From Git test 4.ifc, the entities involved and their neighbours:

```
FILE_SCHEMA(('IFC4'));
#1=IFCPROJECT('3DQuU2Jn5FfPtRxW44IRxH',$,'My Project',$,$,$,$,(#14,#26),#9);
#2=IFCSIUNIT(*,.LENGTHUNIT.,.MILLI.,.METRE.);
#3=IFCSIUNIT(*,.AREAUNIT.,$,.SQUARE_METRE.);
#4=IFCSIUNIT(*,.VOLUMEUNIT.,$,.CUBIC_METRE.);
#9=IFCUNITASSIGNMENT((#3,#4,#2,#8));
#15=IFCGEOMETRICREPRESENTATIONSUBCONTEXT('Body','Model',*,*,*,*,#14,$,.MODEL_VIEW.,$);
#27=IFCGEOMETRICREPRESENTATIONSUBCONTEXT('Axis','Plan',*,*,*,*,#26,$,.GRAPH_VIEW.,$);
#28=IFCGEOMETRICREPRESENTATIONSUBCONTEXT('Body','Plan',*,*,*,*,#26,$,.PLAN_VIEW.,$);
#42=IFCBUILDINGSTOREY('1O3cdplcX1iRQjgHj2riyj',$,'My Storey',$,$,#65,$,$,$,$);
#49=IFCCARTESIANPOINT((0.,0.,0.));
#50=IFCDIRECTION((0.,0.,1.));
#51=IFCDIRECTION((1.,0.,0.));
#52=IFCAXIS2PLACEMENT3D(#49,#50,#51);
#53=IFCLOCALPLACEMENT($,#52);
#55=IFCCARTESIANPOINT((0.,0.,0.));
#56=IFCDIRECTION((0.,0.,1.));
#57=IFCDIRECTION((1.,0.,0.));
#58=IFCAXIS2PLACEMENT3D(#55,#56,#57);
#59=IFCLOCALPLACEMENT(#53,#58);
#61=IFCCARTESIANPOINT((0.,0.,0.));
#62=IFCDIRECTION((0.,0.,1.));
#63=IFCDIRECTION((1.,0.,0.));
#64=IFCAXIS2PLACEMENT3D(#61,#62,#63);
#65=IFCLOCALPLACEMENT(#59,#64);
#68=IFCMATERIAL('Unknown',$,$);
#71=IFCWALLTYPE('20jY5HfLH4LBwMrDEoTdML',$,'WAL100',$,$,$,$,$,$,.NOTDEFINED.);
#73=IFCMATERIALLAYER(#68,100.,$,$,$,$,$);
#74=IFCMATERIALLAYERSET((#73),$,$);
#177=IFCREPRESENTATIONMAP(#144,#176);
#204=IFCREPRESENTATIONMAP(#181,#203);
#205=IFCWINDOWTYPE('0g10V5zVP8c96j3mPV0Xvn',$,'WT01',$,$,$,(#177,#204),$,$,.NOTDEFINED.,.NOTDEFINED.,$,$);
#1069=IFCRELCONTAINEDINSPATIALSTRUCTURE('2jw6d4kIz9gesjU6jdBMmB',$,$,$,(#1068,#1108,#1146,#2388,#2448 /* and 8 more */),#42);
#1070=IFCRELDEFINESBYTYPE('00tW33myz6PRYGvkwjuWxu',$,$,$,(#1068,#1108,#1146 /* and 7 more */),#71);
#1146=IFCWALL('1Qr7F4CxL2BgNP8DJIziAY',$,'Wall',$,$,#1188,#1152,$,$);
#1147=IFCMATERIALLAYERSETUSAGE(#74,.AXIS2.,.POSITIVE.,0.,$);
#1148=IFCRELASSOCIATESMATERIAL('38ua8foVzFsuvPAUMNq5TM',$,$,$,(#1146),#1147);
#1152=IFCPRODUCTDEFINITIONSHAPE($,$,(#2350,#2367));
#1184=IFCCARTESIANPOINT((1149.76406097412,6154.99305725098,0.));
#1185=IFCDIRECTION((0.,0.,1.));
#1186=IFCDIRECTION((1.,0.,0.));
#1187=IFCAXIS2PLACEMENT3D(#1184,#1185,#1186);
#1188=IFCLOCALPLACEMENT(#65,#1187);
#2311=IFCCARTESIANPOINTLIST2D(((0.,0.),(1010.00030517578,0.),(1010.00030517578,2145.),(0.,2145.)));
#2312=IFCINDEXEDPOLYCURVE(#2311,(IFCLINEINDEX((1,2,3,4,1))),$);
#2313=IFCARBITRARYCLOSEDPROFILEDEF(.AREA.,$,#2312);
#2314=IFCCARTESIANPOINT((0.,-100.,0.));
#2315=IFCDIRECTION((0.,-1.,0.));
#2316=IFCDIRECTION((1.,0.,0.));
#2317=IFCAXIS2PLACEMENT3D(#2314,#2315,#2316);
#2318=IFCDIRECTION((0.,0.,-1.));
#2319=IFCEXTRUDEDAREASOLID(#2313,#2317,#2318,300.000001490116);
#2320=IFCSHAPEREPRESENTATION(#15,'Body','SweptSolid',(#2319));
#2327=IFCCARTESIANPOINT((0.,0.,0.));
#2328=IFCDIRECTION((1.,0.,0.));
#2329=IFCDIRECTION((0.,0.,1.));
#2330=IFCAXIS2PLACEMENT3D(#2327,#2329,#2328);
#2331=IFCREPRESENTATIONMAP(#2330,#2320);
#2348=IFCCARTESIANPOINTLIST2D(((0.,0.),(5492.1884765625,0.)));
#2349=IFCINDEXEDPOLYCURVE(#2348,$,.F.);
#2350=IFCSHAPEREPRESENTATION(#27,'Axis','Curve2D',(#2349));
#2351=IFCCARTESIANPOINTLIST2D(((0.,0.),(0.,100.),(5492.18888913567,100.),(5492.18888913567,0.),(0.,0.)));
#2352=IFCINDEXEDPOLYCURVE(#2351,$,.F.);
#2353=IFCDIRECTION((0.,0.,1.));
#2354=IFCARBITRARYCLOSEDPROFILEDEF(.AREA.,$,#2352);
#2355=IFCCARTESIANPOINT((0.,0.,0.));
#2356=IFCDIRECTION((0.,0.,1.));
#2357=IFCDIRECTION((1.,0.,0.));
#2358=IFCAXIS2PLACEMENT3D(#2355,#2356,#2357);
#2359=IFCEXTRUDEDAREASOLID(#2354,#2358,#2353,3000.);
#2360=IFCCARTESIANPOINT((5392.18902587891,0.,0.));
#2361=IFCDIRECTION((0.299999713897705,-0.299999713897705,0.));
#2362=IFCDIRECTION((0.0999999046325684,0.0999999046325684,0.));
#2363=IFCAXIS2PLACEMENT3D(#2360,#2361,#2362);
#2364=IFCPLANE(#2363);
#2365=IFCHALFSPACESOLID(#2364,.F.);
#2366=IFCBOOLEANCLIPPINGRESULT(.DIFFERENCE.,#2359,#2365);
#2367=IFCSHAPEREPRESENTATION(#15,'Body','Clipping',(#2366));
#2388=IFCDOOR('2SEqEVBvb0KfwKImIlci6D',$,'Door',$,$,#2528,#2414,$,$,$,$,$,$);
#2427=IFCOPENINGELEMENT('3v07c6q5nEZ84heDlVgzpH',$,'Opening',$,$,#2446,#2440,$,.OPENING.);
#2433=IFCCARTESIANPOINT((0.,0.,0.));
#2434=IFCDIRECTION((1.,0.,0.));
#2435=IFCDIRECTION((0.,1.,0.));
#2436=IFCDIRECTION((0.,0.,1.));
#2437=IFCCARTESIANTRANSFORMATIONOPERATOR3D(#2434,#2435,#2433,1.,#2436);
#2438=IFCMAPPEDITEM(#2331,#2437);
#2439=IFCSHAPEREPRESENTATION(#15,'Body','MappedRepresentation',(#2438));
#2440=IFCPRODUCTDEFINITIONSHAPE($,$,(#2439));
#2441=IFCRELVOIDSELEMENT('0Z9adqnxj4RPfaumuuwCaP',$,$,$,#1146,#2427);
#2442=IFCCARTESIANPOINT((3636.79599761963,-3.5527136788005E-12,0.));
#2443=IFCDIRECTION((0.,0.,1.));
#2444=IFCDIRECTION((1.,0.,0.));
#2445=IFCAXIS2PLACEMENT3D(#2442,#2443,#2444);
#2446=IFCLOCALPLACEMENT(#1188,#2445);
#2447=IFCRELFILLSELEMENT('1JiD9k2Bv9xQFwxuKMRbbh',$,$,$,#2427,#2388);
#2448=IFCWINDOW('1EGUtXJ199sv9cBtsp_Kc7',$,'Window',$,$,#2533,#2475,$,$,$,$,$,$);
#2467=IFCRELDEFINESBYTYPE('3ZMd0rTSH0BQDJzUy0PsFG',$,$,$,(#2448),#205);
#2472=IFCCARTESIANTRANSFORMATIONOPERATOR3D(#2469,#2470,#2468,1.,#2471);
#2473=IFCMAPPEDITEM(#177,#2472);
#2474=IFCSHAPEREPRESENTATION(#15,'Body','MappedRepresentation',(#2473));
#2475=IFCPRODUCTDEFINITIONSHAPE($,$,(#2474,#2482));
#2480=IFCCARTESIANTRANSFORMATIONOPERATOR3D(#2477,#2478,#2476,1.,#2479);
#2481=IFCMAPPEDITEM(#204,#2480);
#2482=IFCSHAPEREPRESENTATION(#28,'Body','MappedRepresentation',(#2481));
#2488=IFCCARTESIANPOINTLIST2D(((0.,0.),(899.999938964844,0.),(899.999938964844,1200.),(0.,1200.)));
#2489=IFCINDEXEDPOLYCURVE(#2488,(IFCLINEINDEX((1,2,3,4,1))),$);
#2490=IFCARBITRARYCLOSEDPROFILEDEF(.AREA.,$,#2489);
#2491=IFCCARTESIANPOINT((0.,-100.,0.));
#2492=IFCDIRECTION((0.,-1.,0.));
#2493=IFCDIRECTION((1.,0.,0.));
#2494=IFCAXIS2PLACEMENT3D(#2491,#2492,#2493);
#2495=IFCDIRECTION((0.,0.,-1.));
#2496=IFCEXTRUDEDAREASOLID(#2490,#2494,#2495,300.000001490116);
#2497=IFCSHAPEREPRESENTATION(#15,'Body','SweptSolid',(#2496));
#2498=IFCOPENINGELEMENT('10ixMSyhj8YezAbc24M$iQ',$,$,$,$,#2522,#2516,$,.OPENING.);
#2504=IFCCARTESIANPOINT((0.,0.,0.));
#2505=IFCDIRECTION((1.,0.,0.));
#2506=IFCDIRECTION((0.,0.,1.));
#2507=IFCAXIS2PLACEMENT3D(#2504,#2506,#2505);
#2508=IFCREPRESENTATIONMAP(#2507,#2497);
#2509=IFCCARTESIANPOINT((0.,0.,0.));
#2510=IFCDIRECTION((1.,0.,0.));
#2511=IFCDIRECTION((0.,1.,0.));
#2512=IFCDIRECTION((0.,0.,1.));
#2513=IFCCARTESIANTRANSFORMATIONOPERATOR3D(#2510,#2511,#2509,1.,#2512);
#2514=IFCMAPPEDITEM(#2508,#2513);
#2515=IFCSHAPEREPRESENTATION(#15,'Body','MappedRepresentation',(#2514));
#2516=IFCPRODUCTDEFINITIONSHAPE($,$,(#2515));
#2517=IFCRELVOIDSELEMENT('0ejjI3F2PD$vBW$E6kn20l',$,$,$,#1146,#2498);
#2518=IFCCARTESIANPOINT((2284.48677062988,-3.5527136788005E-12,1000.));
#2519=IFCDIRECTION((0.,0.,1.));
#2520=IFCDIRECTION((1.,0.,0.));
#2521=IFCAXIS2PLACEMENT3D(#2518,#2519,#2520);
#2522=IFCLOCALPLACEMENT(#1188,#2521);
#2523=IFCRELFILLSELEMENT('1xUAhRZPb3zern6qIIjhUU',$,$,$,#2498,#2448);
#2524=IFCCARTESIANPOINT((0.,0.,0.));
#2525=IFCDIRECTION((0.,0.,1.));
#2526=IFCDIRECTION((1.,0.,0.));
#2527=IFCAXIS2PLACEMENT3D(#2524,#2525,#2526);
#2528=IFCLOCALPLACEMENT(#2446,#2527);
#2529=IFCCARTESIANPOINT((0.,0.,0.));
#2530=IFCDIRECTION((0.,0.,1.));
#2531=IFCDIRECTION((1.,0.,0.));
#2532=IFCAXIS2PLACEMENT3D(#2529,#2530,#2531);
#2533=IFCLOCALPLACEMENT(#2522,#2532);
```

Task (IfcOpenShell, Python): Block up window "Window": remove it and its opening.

```python
import ifcopenshell
import ifcopenshell.api.feature
import ifcopenshell.api.root
import ifcopenshell.geom
import ifcopenshell.util.shape

model = ifcopenshell.open("Git test 4.ifc")
settings = ifcopenshell.geom.settings()


def volume(element):
    """Net volume in cubic metres, openings subtracted."""
    shape = ifcopenshell.geom.create_shape(settings, element)
    return ifcopenshell.util.shape.get_volume(shape.geometry)


window = model.by_guid("1EGUtXJ199sv9cBtsp_Kc7")
opening = window.FillsVoids[0].RelatingOpeningElement
wall = opening.VoidsElements[0].RelatingBuildingElement
before = volume(wall)

ifcopenshell.api.root.remove_product(model, product=window)
ifcopenshell.api.feature.remove_feature(model, feature=opening)

after = volume(wall)

print(f"wall volume {before:.3f} -> {after:.3f} m3")

model.write("Git test 4_rev.ifc")
```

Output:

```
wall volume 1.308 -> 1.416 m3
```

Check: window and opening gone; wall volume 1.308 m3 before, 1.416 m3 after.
